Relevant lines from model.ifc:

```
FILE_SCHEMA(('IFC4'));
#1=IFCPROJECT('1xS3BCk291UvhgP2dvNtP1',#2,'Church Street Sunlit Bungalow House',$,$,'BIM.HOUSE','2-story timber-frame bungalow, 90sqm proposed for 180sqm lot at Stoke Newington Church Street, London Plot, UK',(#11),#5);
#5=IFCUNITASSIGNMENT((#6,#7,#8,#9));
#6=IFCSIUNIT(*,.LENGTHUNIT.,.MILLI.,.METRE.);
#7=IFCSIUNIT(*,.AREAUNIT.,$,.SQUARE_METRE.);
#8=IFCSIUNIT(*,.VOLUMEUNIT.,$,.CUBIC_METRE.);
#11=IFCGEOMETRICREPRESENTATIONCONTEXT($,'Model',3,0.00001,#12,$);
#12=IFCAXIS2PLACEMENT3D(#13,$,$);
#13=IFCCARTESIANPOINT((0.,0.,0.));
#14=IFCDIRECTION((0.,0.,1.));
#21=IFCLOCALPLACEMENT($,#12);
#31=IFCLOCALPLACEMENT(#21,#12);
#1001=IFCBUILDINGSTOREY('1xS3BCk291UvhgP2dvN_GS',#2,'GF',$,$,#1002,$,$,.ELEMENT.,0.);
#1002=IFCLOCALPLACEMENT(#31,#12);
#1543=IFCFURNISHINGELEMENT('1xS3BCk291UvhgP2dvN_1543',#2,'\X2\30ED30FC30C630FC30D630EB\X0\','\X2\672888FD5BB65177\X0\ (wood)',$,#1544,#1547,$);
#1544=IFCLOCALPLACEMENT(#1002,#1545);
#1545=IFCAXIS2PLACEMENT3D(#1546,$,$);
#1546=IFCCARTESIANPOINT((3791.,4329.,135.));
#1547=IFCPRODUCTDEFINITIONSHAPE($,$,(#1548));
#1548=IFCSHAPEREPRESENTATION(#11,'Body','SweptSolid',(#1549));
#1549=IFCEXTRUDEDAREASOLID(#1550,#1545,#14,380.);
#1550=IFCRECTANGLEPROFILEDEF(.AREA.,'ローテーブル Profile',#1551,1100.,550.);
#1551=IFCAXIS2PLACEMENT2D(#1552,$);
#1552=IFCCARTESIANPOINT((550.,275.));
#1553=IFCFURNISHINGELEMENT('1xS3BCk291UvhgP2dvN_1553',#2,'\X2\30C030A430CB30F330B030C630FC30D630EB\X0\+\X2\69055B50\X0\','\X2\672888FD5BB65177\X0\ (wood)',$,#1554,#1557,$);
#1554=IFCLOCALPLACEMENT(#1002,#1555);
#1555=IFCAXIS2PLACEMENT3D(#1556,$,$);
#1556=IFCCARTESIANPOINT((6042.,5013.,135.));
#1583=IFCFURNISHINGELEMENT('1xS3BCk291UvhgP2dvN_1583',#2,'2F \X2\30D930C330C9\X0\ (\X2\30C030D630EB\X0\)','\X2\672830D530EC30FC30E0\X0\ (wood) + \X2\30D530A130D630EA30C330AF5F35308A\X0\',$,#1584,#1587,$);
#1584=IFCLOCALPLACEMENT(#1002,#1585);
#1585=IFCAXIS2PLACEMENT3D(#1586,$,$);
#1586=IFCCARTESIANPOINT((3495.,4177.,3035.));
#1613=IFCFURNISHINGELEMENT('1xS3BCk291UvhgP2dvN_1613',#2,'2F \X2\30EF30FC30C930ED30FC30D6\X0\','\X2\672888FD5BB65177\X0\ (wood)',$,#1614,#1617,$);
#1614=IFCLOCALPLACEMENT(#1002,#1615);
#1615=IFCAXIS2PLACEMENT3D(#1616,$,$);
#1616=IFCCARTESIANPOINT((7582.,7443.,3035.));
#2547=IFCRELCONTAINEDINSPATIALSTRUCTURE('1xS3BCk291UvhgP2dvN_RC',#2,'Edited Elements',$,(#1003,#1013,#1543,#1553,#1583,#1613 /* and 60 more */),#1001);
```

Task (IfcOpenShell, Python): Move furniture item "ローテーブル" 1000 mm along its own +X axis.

```python
import ifcopenshell
import ifcopenshell.api.geometry
import ifcopenshell.util.placement
import ifcopenshell.util.unit

model = ifcopenshell.open("model.ifc")
unit_scale = ifcopenshell.util.unit.calculate_unit_scale(model)

item = model.by_guid("1xS3BCk291UvhgP2dvN_1543")
matrix = ifcopenshell.util.placement.get_local_placement(item.ObjectPlacement)
matrix[:3, 3] += matrix[:3, 0] * 1 / unit_scale
ifcopenshell.api.geometry.edit_object_placement(model, product=item, matrix=matrix, is_si=False)

print(ifcopenshell.util.placement.get_local_placement(item.ObjectPlacement).round(3) + 0.0)

model.write("model-out.ifc")
```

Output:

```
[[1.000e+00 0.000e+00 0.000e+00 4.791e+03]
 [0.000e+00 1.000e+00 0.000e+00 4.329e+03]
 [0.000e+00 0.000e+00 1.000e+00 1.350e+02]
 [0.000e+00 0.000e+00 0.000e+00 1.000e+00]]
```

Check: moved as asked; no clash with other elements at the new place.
